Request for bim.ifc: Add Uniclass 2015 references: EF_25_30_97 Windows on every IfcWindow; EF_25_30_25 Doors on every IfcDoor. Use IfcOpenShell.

First a look at what the model holds.

```python
import ifcopenshell

model = ifcopenshell.open("bim.ifc")
print(model.schema)
print("classifications:", [c.Name for c in model.by_type("IfcClassification")])
for ifc_class in ("IfcDoor", "IfcRoof", "IfcStair", "IfcWall", "IfcWindow"):
    print(ifc_class, len(model.by_type(ifc_class)))
```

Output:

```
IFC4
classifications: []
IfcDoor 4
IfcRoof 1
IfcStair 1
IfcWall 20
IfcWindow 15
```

```python
import ifcopenshell
import ifcopenshell.api.classification

model = ifcopenshell.open("bim.ifc")

system = ifcopenshell.api.classification.add_classification(model, classification="Uniclass 2015")

codes = {
    "IfcWindow": ("EF_25_30_97", "Windows"),
    "IfcDoor": ("EF_25_30_25", "Doors"),
}
for ifc_class, (code, name) in codes.items():
    products = model.by_type(ifc_class)
    ifcopenshell.api.classification.add_reference(
        model, products=products, classification=system, identification=code, name=name
    )
    print(code, len(products))

model.write("bim_updated.ifc")
```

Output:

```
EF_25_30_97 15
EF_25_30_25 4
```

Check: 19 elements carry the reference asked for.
